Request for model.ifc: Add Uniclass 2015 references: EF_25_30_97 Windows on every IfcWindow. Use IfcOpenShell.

First a look at what the model holds.

```python
import ifcopenshell

model = ifcopenshell.open("model.ifc")
print(model.schema)
print("classifications:", [c.Name for c in model.by_type("IfcClassification")])
for ifc_class in ("IfcDoor", "IfcRoof", "IfcStair", "IfcWall", "IfcWindow"):
    print(ifc_class, len(model.by_type(ifc_class)))
```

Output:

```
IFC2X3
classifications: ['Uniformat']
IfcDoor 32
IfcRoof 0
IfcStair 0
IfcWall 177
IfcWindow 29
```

```python
import ifcopenshell
import ifcopenshell.api.classification

model = ifcopenshell.open("model.ifc")

# IFC2X3 requires Source and Edition and has no link from the project to the system.
system = model.create_entity("IfcClassification", Source="NBS", Edition="2015", Name="Uniclass 2015")

codes = {
    "IfcWindow": ("EF_25_30_97", "Windows"),
}
for ifc_class, (code, name) in codes.items():
    products = model.by_type(ifc_class)
    ifcopenshell.api.classification.add_reference(
        model, products=products, classification=system, identification=code, name=name
    )
    print(code, len(products))

model.write("model_updated.ifc")
```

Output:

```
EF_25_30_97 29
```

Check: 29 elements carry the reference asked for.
